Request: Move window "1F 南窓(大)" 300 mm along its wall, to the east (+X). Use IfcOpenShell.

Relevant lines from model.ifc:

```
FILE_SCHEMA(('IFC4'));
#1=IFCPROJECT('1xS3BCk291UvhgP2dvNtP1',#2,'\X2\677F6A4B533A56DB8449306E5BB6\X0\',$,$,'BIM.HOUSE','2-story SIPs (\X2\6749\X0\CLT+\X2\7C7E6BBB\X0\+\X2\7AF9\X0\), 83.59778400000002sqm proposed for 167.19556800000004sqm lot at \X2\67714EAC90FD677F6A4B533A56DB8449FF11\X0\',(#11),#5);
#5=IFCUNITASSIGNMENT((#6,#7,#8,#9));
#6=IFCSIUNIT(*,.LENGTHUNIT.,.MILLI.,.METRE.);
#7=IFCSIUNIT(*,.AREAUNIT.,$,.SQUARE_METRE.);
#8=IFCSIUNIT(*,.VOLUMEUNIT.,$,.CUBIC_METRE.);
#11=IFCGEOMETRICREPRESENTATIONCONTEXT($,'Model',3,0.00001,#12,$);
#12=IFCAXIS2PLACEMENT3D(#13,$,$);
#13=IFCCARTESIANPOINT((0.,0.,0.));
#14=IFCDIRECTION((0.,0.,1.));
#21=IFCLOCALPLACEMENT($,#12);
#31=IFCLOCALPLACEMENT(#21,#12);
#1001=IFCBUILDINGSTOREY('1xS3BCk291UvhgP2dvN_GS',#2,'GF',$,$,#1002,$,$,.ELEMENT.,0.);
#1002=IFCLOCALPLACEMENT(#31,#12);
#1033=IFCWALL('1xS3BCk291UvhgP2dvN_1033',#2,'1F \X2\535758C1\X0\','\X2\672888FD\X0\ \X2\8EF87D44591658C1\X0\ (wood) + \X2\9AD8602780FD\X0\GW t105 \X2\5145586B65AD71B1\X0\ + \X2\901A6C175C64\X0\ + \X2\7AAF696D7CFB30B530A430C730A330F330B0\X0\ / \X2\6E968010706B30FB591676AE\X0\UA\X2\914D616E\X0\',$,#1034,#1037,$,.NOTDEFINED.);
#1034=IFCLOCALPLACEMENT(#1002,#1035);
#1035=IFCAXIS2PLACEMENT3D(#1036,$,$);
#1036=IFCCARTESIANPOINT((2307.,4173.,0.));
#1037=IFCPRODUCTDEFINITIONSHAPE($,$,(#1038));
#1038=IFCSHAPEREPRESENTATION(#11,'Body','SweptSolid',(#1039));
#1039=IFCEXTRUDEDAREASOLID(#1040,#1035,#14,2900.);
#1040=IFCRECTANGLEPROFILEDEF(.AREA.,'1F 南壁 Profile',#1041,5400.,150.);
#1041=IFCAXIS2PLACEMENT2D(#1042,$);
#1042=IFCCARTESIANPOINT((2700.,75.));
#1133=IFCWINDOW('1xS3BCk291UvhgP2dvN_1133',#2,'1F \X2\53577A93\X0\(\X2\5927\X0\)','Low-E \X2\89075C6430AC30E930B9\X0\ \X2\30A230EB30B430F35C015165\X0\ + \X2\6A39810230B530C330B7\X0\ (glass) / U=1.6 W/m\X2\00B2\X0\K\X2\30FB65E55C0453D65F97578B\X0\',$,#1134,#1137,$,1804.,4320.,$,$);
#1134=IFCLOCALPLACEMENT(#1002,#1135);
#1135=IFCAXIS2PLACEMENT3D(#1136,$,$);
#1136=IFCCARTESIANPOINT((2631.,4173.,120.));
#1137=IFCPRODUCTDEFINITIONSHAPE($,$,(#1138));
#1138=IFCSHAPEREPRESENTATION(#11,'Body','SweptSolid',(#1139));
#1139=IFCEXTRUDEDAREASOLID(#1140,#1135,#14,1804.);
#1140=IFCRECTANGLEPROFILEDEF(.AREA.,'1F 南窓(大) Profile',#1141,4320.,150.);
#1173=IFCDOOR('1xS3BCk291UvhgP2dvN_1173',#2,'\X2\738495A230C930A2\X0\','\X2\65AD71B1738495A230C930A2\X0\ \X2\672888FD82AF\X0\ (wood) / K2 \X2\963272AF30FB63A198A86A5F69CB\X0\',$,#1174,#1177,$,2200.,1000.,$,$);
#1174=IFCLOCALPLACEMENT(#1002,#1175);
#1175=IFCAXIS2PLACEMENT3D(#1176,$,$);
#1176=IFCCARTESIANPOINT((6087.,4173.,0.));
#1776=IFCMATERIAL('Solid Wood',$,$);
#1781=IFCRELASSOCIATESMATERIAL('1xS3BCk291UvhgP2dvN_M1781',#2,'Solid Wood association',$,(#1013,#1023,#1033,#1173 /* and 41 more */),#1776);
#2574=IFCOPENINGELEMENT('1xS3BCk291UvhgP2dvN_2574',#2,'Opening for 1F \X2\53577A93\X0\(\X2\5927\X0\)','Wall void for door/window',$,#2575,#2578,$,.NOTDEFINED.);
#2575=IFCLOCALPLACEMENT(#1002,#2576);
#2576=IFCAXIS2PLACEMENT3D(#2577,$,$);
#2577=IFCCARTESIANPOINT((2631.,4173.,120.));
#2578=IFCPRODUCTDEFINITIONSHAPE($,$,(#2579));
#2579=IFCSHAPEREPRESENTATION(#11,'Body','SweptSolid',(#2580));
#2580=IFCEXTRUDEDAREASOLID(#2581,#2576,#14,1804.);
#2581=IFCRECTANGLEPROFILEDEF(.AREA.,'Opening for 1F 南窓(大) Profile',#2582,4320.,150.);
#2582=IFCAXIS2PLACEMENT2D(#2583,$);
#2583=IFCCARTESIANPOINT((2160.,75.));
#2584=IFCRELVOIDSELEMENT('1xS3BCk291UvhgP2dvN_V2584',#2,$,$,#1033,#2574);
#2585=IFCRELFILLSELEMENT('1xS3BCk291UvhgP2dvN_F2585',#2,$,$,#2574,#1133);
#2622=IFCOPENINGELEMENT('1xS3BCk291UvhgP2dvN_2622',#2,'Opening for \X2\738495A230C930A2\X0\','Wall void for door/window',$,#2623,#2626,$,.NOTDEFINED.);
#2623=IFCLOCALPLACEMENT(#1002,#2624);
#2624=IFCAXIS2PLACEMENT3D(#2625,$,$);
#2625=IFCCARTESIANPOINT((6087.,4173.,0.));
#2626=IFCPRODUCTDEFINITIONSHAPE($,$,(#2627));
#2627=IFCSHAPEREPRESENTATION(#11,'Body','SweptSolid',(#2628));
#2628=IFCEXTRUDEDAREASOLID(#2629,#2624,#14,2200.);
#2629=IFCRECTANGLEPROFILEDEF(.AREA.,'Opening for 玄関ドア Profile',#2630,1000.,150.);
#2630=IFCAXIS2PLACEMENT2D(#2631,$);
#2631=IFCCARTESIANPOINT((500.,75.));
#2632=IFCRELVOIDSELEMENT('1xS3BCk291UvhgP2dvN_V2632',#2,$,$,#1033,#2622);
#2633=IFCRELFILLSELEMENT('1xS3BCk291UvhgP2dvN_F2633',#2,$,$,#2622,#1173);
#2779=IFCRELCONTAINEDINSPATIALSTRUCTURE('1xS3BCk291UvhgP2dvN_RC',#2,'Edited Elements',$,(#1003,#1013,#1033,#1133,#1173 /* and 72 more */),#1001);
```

```python
import ifcopenshell
import ifcopenshell.api.geometry
import ifcopenshell.util.placement

model = ifcopenshell.open("model.ifc")

window = model.by_guid("1xS3BCk291UvhgP2dvN_1133")
opening = window.FillsVoids[0].RelatingOpeningElement
wall = opening.VoidsElements[0].RelatingBuildingElement

wall_matrix = ifcopenshell.util.placement.get_local_placement(wall.ObjectPlacement)
shift = wall_matrix[:3, 0] * 300.0
before = ifcopenshell.util.placement.get_local_placement(window.ObjectPlacement)[:3, 3].copy()

# The window is not placed relative to its opening, so move both.
for product in (opening, window):
    matrix = ifcopenshell.util.placement.get_local_placement(product.ObjectPlacement)
    matrix[:3, 3] += shift
    ifcopenshell.api.geometry.edit_object_placement(model, product=product, matrix=matrix, is_si=False)

after = ifcopenshell.util.placement.get_local_placement(window.ObjectPlacement)[:3, 3]
print("window moved by", (after - before).round(3) + 0.0)

model.write("model-out.ifc")
```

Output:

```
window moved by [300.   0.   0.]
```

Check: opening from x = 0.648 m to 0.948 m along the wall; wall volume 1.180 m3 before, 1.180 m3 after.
